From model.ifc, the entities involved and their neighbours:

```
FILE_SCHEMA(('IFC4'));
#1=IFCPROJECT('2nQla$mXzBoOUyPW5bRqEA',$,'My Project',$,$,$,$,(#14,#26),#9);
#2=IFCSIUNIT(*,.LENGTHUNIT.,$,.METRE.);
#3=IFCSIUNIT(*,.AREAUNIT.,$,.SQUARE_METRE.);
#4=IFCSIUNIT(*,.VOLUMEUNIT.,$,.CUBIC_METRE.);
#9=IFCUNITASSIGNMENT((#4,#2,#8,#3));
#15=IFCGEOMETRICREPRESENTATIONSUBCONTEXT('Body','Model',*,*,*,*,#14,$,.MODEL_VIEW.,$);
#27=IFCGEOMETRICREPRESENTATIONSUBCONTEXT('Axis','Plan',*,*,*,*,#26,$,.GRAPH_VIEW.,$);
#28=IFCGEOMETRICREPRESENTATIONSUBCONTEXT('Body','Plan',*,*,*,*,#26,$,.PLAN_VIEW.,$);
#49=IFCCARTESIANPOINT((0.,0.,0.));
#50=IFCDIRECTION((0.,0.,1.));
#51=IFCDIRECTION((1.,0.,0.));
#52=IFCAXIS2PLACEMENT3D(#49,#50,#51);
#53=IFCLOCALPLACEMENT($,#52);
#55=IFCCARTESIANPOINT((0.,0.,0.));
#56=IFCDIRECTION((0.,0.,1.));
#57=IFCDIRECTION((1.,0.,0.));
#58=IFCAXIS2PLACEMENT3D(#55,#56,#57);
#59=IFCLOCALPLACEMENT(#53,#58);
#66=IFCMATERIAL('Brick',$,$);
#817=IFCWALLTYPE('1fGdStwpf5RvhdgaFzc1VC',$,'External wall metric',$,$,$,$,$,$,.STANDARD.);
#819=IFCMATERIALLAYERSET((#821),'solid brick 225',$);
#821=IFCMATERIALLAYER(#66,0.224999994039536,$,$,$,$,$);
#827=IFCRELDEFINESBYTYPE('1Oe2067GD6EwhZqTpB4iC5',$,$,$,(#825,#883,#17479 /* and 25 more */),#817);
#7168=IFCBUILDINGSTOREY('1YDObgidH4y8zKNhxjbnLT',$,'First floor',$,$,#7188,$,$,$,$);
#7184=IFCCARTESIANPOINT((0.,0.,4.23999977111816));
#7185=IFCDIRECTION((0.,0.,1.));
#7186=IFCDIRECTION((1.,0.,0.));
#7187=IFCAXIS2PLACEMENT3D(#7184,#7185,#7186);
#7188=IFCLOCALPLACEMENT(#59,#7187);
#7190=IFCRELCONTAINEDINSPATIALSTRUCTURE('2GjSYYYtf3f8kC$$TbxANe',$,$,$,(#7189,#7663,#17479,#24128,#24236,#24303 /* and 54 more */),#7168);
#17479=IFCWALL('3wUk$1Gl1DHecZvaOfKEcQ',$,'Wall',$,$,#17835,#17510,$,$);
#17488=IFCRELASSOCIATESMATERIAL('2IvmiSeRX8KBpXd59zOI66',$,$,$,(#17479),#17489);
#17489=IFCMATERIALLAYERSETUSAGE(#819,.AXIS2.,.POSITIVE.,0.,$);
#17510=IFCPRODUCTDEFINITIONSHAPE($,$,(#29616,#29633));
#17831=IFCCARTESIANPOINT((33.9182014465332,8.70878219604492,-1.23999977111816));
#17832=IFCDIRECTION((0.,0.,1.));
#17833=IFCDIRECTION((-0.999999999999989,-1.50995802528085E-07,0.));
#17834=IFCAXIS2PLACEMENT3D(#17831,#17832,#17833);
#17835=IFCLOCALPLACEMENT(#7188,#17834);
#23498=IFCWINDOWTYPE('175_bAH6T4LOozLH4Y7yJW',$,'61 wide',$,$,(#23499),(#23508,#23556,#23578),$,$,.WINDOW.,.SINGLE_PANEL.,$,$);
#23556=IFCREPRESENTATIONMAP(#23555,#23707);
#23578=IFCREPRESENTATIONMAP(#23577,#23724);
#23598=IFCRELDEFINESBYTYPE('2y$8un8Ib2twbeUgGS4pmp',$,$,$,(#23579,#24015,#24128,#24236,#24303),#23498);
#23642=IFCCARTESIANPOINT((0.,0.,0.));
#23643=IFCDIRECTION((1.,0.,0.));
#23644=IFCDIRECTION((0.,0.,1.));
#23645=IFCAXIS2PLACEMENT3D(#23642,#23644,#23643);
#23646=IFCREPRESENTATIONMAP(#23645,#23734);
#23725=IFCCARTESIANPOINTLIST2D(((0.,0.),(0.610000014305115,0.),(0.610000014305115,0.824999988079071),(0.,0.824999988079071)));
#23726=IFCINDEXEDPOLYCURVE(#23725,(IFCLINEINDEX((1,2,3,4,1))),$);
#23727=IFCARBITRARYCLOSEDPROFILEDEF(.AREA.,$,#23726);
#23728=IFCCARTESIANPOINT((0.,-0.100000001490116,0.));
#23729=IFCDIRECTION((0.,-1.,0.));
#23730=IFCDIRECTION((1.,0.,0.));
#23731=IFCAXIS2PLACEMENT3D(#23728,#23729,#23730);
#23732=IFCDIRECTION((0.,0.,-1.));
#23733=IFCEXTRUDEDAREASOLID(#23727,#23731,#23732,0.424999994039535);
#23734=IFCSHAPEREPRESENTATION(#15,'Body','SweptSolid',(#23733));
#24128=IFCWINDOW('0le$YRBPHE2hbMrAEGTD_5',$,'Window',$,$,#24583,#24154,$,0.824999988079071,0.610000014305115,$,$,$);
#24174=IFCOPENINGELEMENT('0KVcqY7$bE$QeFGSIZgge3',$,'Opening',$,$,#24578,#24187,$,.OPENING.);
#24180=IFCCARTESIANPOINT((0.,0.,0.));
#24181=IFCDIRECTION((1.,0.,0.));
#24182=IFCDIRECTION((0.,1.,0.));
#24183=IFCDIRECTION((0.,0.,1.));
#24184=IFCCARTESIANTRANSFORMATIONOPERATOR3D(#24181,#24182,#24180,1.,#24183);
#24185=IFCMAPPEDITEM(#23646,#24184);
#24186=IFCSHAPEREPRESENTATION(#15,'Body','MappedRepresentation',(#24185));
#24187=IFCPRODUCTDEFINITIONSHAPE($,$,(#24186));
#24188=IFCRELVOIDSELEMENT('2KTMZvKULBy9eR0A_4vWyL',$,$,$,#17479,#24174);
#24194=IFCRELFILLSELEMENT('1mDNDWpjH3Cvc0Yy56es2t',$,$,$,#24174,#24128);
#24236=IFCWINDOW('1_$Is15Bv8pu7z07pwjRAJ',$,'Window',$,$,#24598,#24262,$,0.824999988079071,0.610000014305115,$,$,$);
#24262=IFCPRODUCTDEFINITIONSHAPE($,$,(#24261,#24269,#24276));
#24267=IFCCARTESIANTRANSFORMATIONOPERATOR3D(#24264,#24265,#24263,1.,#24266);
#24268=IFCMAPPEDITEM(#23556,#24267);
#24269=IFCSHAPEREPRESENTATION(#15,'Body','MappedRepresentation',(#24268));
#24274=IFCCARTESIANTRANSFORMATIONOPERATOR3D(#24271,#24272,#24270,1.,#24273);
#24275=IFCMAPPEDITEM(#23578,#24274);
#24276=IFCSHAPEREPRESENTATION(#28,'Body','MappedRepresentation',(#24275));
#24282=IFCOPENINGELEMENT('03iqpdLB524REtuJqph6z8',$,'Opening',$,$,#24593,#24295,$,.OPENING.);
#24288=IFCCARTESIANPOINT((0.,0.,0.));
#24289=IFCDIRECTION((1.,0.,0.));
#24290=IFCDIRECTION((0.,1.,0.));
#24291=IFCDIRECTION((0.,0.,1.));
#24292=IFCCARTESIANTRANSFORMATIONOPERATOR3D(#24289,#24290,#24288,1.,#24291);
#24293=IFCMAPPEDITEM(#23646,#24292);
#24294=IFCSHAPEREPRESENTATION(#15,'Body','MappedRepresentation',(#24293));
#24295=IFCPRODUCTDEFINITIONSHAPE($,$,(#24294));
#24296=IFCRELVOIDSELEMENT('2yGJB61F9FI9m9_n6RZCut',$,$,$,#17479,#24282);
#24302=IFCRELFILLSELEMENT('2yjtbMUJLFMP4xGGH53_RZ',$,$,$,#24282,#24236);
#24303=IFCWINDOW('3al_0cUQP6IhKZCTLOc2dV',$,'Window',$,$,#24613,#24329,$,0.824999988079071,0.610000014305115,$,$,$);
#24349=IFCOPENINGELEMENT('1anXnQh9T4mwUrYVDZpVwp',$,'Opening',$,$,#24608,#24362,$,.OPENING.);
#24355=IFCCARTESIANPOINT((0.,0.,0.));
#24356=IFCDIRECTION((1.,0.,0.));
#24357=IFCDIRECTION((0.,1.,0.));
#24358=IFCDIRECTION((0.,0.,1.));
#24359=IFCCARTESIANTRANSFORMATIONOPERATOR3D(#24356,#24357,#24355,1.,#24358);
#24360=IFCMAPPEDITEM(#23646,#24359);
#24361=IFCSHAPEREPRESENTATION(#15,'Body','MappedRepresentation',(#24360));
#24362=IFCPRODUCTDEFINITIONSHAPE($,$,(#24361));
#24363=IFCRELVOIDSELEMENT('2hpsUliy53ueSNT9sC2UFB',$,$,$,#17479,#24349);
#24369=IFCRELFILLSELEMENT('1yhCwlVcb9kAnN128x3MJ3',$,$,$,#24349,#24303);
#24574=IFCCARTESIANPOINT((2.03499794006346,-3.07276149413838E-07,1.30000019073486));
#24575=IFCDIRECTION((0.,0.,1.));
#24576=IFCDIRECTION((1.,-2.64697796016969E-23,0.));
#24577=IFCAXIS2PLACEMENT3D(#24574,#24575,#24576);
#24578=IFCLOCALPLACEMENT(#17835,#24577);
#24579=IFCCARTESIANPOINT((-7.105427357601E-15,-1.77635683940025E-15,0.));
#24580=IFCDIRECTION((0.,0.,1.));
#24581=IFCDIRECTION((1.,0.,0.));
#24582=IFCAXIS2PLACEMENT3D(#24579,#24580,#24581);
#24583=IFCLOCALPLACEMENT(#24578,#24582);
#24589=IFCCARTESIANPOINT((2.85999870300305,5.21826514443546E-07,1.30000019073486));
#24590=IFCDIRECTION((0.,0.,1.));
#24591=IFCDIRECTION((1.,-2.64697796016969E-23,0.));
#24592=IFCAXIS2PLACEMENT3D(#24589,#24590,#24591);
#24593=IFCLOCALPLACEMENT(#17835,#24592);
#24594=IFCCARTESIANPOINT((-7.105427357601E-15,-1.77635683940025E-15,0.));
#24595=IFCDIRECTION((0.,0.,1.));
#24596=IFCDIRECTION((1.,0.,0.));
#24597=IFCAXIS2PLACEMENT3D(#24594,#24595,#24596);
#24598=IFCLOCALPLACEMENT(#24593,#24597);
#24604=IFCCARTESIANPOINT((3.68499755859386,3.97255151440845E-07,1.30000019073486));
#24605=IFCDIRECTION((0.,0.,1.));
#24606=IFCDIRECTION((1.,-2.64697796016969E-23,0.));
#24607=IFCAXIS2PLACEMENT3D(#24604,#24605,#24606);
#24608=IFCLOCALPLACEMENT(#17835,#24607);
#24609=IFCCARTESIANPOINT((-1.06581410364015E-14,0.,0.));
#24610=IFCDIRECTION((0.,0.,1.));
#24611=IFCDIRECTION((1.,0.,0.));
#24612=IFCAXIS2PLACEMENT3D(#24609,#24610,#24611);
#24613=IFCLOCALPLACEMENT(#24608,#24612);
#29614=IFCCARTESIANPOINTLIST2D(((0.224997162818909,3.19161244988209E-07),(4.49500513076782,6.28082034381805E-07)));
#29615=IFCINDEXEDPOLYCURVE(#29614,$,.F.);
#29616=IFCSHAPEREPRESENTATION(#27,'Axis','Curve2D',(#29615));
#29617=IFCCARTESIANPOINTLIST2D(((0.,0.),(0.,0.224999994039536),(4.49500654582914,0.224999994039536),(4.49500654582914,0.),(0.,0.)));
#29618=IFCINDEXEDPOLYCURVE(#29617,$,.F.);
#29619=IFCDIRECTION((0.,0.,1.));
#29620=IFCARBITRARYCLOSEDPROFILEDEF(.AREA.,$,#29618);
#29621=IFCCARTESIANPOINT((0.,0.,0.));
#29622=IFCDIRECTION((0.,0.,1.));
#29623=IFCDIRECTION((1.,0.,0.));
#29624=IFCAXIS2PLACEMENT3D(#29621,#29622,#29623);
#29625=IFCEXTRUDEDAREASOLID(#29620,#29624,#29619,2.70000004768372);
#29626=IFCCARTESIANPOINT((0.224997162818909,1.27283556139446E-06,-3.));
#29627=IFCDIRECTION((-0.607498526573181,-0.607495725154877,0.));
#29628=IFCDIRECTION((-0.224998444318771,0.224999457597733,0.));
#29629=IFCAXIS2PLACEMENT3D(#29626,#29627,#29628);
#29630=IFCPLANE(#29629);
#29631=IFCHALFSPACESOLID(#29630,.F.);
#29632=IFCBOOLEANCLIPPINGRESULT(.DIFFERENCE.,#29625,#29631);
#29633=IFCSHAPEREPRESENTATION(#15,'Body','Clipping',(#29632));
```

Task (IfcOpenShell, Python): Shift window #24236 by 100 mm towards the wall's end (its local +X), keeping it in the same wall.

```python
import ifcopenshell
import ifcopenshell.api.geometry
import ifcopenshell.util.placement
import ifcopenshell.util.unit

model = ifcopenshell.open("model.ifc")
unit_scale = ifcopenshell.util.unit.calculate_unit_scale(model)

window = model.by_guid("1_$Is15Bv8pu7z07pwjRAJ")
opening = window.FillsVoids[0].RelatingOpeningElement
wall = opening.VoidsElements[0].RelatingBuildingElement

wall_matrix = ifcopenshell.util.placement.get_local_placement(wall.ObjectPlacement)
shift = wall_matrix[:3, 0] * 0.1 / unit_scale
before = ifcopenshell.util.placement.get_local_placement(window.ObjectPlacement)[:3, 3].copy()

# The window is placed relative to its opening, so it follows when the opening moves.
matrix = ifcopenshell.util.placement.get_local_placement(opening.ObjectPlacement)
matrix[:3, 3] += shift
ifcopenshell.api.geometry.edit_object_placement(
    model, product=opening, matrix=matrix, is_si=False, should_transform_children=True
)

after = ifcopenshell.util.placement.get_local_placement(window.ObjectPlacement)[:3, 3]
print("window moved by", (after - before).round(3) + 0.0)

model.write("model_v2.ifc")
```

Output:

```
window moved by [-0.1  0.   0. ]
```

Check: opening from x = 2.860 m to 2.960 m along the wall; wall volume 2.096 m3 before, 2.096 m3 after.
